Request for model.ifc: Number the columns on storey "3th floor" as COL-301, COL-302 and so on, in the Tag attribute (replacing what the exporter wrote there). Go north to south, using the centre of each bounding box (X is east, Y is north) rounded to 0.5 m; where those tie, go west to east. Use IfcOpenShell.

First a look at what the model holds.

```python
import ifcopenshell
import ifcopenshell.util.element
import ifcopenshell.util.placement

model = ifcopenshell.open("model.ifc")
print(model.schema)
storey = next(s for s in model.by_type("IfcBuildingStorey") if s.Name == "3th floor")
columns = [e for e in ifcopenshell.util.element.get_decomposition(storey) if e.is_a("IfcColumn")]
for e in sorted(columns, key=lambda e: e.id()):
    origin = ifcopenshell.util.placement.get_local_placement(e.ObjectPlacement)[:3, 3]
    print(e.id(), e.Tag, e.Name, origin.round(2) + 0.0, sep=" | ")
```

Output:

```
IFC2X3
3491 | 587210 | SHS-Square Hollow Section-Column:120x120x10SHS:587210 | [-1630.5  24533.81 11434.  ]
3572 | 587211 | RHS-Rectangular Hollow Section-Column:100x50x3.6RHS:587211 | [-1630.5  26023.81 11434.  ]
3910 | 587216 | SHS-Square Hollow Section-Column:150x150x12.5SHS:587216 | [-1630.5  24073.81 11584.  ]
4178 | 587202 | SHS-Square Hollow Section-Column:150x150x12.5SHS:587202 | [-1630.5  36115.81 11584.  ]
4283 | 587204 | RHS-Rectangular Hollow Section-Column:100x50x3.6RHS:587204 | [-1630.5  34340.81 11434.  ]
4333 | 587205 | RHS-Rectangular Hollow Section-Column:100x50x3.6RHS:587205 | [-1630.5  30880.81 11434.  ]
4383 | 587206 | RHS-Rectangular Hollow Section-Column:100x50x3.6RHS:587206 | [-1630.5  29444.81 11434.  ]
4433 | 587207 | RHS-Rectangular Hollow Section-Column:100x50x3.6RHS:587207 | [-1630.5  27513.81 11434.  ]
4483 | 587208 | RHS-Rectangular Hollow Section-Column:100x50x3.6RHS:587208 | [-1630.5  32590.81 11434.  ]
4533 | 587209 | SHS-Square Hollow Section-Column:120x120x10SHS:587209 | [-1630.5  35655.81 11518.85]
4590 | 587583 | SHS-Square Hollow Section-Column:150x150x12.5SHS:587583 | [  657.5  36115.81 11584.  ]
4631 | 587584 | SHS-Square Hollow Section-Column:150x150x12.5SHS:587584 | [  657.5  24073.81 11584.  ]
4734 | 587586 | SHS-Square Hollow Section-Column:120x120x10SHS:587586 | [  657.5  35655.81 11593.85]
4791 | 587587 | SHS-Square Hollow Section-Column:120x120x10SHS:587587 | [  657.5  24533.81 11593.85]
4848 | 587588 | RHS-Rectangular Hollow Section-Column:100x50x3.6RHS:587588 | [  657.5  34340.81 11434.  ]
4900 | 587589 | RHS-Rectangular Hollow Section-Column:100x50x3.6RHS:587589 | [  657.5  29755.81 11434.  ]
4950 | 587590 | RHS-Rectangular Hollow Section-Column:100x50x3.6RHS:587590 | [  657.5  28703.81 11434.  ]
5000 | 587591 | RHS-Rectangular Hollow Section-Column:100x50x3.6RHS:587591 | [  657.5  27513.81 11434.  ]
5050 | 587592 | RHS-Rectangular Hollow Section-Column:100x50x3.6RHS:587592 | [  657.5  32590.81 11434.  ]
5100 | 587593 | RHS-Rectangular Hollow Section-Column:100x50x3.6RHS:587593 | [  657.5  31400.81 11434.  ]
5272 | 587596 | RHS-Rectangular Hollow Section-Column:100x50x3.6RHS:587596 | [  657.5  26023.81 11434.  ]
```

```python
import ifcopenshell
import ifcopenshell.geom
import ifcopenshell.util.element
import ifcopenshell.util.shape

model = ifcopenshell.open("model.ifc")
settings = ifcopenshell.geom.settings()
settings.set("use-world-coords", True)


def centre(element):
    shape = ifcopenshell.geom.create_shape(settings, element)
    return ifcopenshell.util.shape.get_bbox_centroid(shape.geometry)


storey = next(s for s in model.by_type("IfcBuildingStorey") if s.Name == "3th floor")
columns = [e for e in ifcopenshell.util.element.get_decomposition(storey) if e.is_a("IfcColumn")]

# Insertion points can sit at a corner or the storey origin, so sort by the geometry (in metres).
centres = {e: centre(e) for e in columns}
columns.sort(key=lambda e: (-round(centres[e][1] / 0.5), centres[e][0]))

for i, e in enumerate(columns, start=1):
    number = f"COL-3{i:02d}"
    e.Tag = number
    print(e.id(), number)

model.write("model_updated.ifc")
```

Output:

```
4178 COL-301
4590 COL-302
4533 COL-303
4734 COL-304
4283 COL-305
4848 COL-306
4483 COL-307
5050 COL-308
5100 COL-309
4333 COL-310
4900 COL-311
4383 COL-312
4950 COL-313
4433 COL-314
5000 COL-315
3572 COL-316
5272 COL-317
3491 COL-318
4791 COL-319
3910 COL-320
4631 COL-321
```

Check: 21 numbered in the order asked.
